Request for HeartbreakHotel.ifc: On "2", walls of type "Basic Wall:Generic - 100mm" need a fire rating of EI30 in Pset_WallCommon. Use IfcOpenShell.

First a look at what the model holds.

```python
import ifcopenshell
import ifcopenshell.util.element

model = ifcopenshell.open("HeartbreakHotel.ifc")
print(model.schema)
storey = next(s for s in model.by_type("IfcBuildingStorey") if s.Name == "2")
walls = [e for e in ifcopenshell.util.element.get_decomposition(storey) if e.is_a("IfcWall")]
seen = {}
for e in walls:
    element_type = ifcopenshell.util.element.get_type(e)
    key = (element_type.Name if element_type != e and element_type else None, ifcopenshell.util.element.get_pset(e, "Pset_WallCommon", "FireRating"))
    seen[key] = seen.get(key, 0) + 1
for (name, value), count in sorted(seen.items(), key=str):
    print(count, "x", name, "|", value)
```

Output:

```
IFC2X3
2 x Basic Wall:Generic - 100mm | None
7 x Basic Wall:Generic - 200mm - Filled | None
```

```python
import ifcopenshell
import ifcopenshell.api.pset
import ifcopenshell.util.element

model = ifcopenshell.open("HeartbreakHotel.ifc")

storey = next(s for s in model.by_type("IfcBuildingStorey") if s.Name == "2")
walls = [e for e in ifcopenshell.util.element.get_decomposition(storey) if e.is_a("IfcWall")]

count = 0
for e in walls:
    element_type = ifcopenshell.util.element.get_type(e)
    if element_type in (None, e) or element_type.Name != "Basic Wall:Generic - 100mm":
        continue
    # add_pset returns the element's existing set when there is one.
    pset = ifcopenshell.api.pset.add_pset(model, product=e, name="Pset_WallCommon")
    ifcopenshell.api.pset.edit_pset(model, pset=pset, properties={"FireRating": "EI30"})
    count += 1

print(count, "walls updated")

model.write("HeartbreakHotel_rev.ifc")
```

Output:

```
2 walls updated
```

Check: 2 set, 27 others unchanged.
